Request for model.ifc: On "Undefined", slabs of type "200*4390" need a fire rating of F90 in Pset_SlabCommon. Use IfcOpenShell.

First a look at what the model holds.

```python
import ifcopenshell
import ifcopenshell.util.element

model = ifcopenshell.open("model.ifc")
print(model.schema)
storey = next(s for s in model.by_type("IfcBuildingStorey") if s.Name == "Undefined")
slabs = [e for e in ifcopenshell.util.element.get_decomposition(storey) if e.is_a("IfcSlab")]
seen = {}
for e in slabs:
    element_type = ifcopenshell.util.element.get_type(e)
    key = (element_type.Name if element_type != e and element_type else None, ifcopenshell.util.element.get_pset(e, "Pset_SlabCommon", "FireRating"))
    seen[key] = seen.get(key, 0) + 1
for (name, value), count in sorted(seen.items(), key=str):
    print(count, "x", name, "|", value)
```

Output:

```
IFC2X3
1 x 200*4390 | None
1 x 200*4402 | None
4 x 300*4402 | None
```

```python
import ifcopenshell
import ifcopenshell.api.pset
import ifcopenshell.util.element

model = ifcopenshell.open("model.ifc")

storey = next(s for s in model.by_type("IfcBuildingStorey") if s.Name == "Undefined")
slabs = [e for e in ifcopenshell.util.element.get_decomposition(storey) if e.is_a("IfcSlab")]

count = 0
for e in slabs:
    element_type = ifcopenshell.util.element.get_type(e)
    if element_type in (None, e) or element_type.Name != "200*4390":
        continue
    # add_pset returns the element's existing set when there is one.
    pset = ifcopenshell.api.pset.add_pset(model, product=e, name="Pset_SlabCommon")
    ifcopenshell.api.pset.edit_pset(model, pset=pset, properties={"FireRating": "F90"})
    count += 1

print(count, "slabs updated")

model.write("model_updated.ifc")
```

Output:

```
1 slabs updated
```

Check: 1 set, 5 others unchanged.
